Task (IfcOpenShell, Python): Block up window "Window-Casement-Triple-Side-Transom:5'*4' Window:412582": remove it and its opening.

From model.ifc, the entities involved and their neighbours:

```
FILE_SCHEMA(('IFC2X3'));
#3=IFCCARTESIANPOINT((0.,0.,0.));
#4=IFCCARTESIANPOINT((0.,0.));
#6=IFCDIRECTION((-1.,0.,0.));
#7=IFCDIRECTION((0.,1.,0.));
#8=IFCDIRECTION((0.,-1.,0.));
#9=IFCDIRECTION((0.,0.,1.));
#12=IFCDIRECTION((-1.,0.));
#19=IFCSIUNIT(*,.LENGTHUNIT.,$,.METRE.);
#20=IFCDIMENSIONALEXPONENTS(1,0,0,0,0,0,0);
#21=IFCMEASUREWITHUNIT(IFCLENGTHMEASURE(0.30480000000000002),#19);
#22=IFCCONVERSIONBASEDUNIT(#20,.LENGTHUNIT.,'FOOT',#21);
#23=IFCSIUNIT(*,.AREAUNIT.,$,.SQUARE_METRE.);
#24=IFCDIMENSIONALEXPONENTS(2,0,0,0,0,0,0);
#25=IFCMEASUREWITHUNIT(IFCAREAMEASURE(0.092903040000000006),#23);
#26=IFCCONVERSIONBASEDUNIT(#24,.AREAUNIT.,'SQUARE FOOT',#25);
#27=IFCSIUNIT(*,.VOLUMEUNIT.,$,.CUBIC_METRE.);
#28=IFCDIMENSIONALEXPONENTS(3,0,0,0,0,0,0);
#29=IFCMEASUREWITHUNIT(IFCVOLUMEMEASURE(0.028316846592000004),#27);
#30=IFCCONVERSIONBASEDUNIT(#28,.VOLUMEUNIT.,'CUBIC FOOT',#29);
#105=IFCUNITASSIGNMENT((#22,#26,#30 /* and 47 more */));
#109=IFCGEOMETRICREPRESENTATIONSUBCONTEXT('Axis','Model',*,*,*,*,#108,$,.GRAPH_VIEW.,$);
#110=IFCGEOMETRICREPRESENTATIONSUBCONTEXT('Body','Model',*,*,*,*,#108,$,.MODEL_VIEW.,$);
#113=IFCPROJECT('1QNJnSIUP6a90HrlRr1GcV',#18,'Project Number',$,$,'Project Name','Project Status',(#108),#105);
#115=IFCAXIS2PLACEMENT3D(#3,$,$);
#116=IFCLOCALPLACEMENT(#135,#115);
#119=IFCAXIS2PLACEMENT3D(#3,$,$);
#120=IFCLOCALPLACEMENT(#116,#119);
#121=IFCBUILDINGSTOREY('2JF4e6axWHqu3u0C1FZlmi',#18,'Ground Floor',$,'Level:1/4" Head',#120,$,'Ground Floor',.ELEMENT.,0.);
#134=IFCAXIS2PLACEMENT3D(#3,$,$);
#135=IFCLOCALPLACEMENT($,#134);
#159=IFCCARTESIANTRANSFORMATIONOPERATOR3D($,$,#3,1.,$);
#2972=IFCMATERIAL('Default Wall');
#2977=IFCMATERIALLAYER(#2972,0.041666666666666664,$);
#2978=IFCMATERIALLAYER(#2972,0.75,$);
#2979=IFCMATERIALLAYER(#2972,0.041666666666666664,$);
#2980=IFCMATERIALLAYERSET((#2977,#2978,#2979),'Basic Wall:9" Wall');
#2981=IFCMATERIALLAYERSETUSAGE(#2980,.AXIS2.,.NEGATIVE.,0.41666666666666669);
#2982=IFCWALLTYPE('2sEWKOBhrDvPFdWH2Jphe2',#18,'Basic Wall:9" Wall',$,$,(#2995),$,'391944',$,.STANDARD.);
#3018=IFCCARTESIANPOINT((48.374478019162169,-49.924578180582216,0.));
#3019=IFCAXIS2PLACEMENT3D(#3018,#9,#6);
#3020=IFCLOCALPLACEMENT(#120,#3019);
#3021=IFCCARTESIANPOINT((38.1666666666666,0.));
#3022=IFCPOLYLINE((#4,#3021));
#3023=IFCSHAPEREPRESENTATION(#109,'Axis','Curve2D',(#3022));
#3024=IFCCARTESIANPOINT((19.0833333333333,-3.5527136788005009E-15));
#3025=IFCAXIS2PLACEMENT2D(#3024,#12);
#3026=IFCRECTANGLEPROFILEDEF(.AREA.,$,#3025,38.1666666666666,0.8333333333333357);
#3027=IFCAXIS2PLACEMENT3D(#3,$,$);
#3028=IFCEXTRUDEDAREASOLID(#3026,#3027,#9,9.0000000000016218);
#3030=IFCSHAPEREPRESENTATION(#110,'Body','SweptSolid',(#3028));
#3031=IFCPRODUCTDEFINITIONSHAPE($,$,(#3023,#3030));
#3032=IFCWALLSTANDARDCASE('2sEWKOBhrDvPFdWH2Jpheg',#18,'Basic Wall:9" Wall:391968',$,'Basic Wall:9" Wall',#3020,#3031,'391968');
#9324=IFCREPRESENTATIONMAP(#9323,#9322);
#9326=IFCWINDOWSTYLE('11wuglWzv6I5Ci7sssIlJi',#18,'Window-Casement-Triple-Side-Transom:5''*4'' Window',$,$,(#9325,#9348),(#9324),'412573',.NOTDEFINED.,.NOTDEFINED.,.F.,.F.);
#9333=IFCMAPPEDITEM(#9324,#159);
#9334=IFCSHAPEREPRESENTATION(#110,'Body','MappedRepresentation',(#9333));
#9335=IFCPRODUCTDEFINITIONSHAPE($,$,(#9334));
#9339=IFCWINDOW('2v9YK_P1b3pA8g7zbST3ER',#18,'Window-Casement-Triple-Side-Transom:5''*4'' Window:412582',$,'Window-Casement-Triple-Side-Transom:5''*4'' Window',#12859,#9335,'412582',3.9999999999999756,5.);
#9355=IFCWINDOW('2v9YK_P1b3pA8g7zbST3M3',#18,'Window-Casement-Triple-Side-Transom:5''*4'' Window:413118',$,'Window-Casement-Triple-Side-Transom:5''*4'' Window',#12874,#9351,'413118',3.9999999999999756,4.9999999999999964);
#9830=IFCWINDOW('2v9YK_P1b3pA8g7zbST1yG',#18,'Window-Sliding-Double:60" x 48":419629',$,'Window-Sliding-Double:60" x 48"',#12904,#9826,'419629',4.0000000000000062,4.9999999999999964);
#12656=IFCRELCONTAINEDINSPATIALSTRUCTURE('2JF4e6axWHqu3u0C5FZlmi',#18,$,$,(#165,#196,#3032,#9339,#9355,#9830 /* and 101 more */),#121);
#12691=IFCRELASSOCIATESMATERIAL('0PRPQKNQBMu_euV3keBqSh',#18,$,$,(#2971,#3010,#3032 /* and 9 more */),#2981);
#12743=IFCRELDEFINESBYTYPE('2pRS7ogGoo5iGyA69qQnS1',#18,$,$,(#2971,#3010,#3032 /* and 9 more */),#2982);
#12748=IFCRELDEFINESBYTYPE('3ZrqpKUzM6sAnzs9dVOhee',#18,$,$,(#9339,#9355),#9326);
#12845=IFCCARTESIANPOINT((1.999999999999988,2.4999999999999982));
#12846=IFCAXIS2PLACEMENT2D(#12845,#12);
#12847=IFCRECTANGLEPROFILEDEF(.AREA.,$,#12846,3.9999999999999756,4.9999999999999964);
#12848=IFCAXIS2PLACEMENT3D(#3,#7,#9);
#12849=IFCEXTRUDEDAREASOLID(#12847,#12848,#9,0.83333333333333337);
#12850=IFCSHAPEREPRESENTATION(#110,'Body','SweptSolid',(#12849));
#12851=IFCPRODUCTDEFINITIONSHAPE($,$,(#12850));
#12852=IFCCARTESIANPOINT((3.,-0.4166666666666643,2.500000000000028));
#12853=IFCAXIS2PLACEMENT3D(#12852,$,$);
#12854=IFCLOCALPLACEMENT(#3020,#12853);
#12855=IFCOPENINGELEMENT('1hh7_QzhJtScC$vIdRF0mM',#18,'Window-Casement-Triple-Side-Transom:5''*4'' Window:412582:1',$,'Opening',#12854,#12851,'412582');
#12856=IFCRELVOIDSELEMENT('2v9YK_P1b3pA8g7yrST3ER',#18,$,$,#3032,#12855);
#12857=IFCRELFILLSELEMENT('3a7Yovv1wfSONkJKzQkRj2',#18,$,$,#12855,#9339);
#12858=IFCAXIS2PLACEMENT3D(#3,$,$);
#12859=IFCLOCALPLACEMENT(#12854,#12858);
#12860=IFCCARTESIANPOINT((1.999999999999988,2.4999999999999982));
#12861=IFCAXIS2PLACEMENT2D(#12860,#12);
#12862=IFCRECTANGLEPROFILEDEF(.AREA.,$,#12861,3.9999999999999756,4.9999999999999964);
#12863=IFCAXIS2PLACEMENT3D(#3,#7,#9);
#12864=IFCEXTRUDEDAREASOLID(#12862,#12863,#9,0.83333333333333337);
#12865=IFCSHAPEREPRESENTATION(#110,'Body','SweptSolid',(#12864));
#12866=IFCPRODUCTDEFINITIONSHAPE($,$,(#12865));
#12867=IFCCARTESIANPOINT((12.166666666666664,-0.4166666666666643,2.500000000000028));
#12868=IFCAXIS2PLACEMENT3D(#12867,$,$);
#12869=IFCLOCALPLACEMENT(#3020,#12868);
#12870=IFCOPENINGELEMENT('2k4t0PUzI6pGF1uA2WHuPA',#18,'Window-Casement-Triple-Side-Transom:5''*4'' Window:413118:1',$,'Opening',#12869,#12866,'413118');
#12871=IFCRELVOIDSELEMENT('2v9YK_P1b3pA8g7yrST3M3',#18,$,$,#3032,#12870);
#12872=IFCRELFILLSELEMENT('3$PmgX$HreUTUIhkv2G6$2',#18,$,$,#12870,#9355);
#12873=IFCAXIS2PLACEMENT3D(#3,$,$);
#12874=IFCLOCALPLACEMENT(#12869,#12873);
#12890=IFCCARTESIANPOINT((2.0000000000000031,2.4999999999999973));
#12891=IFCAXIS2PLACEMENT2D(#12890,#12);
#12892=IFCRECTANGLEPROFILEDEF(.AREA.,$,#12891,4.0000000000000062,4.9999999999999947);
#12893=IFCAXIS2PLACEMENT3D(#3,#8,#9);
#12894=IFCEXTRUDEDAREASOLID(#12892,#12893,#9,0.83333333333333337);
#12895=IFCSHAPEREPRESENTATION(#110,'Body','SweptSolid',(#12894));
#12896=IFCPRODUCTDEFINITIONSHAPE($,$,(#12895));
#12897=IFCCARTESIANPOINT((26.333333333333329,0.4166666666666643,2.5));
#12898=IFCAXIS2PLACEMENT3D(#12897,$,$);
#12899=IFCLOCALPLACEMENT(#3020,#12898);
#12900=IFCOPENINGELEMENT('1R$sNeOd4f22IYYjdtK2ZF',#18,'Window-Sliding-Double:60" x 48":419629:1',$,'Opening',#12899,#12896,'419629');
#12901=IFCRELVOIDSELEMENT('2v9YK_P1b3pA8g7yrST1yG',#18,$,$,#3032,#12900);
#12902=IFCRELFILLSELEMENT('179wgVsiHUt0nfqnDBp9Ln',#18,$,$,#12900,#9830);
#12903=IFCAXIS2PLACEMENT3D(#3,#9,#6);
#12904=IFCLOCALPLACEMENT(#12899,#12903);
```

```python
import ifcopenshell
import ifcopenshell.api.feature
import ifcopenshell.api.root
import ifcopenshell.geom
import ifcopenshell.util.shape

model = ifcopenshell.open("model.ifc")
settings = ifcopenshell.geom.settings()


def volume(element):
    """Net volume in cubic metres, openings subtracted."""
    shape = ifcopenshell.geom.create_shape(settings, element)
    return ifcopenshell.util.shape.get_volume(shape.geometry)


window = model.by_id(9339)
opening = window.FillsVoids[0].RelatingOpeningElement
wall = opening.VoidsElements[0].RelatingBuildingElement
before = volume(wall)

ifcopenshell.api.root.remove_product(model, product=window)
ifcopenshell.api.feature.remove_feature(model, feature=opening)

after = volume(wall)

print(f"wall volume {before:.3f} -> {after:.3f} m3")

model.write("model_rev.ifc")
```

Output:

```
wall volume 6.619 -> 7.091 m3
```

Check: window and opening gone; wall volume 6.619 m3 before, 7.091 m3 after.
